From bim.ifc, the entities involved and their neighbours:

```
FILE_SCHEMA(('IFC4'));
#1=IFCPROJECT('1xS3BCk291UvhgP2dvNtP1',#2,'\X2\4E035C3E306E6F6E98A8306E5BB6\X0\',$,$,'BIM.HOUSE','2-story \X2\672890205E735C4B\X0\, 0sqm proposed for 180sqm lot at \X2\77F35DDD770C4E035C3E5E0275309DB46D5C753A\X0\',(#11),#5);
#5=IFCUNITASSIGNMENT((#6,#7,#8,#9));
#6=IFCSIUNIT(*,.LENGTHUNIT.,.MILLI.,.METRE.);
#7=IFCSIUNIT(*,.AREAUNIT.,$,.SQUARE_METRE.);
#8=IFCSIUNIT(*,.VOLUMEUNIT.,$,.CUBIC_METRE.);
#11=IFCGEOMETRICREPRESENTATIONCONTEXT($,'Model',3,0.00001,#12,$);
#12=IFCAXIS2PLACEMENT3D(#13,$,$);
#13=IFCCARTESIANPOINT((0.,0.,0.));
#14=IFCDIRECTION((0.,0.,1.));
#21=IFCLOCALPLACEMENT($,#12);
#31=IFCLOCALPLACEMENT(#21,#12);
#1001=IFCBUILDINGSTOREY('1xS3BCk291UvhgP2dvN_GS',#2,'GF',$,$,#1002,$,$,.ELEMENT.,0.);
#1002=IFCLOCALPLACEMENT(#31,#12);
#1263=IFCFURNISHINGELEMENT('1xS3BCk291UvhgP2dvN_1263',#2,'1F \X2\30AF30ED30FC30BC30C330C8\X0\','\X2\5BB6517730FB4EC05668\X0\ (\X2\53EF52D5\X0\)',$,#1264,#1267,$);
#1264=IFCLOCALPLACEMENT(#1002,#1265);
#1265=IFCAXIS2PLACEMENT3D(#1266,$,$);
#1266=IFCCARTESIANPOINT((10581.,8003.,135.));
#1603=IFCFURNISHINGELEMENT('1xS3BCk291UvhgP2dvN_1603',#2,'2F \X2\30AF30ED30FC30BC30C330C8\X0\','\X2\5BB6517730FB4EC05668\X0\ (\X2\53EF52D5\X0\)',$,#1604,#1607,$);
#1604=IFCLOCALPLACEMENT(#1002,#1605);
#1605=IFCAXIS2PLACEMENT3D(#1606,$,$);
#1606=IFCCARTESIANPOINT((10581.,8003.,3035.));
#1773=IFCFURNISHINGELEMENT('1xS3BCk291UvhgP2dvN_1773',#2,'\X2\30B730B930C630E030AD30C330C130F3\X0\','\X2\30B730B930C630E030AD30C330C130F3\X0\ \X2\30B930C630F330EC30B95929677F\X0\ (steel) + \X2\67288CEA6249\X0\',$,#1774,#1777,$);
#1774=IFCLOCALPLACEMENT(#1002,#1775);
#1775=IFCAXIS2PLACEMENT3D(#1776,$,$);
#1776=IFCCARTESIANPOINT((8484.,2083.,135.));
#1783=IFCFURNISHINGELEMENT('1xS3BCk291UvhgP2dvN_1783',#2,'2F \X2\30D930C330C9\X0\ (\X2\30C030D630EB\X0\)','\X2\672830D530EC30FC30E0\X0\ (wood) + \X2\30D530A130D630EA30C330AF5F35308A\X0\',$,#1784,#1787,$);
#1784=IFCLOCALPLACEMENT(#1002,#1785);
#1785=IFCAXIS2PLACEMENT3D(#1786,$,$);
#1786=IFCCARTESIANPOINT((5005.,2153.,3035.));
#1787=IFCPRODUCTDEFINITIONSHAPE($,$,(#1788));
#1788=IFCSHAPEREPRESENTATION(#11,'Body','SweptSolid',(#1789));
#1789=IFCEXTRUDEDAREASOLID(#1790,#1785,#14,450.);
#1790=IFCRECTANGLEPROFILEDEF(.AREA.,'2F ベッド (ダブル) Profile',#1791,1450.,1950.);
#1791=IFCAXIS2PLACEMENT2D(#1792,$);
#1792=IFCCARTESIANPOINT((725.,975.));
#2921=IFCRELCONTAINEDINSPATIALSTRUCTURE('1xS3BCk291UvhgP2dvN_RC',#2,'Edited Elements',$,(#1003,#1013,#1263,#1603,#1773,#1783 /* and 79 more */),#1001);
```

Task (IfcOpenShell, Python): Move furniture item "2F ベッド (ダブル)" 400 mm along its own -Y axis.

```python
import ifcopenshell
import ifcopenshell.api.geometry
import ifcopenshell.util.placement

model = ifcopenshell.open("bim.ifc")

item = model.by_guid("1xS3BCk291UvhgP2dvN_1783")
matrix = ifcopenshell.util.placement.get_local_placement(item.ObjectPlacement)
matrix[:3, 3] -= matrix[:3, 1] * 400.0
ifcopenshell.api.geometry.edit_object_placement(model, product=item, matrix=matrix, is_si=False)

print(ifcopenshell.util.placement.get_local_placement(item.ObjectPlacement).round(3) + 0.0)

model.write("bim_updated.ifc")
```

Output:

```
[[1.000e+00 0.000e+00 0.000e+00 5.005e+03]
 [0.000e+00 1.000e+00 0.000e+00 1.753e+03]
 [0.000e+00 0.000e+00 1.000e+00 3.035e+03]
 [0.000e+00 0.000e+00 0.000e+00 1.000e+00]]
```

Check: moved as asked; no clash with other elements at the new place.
